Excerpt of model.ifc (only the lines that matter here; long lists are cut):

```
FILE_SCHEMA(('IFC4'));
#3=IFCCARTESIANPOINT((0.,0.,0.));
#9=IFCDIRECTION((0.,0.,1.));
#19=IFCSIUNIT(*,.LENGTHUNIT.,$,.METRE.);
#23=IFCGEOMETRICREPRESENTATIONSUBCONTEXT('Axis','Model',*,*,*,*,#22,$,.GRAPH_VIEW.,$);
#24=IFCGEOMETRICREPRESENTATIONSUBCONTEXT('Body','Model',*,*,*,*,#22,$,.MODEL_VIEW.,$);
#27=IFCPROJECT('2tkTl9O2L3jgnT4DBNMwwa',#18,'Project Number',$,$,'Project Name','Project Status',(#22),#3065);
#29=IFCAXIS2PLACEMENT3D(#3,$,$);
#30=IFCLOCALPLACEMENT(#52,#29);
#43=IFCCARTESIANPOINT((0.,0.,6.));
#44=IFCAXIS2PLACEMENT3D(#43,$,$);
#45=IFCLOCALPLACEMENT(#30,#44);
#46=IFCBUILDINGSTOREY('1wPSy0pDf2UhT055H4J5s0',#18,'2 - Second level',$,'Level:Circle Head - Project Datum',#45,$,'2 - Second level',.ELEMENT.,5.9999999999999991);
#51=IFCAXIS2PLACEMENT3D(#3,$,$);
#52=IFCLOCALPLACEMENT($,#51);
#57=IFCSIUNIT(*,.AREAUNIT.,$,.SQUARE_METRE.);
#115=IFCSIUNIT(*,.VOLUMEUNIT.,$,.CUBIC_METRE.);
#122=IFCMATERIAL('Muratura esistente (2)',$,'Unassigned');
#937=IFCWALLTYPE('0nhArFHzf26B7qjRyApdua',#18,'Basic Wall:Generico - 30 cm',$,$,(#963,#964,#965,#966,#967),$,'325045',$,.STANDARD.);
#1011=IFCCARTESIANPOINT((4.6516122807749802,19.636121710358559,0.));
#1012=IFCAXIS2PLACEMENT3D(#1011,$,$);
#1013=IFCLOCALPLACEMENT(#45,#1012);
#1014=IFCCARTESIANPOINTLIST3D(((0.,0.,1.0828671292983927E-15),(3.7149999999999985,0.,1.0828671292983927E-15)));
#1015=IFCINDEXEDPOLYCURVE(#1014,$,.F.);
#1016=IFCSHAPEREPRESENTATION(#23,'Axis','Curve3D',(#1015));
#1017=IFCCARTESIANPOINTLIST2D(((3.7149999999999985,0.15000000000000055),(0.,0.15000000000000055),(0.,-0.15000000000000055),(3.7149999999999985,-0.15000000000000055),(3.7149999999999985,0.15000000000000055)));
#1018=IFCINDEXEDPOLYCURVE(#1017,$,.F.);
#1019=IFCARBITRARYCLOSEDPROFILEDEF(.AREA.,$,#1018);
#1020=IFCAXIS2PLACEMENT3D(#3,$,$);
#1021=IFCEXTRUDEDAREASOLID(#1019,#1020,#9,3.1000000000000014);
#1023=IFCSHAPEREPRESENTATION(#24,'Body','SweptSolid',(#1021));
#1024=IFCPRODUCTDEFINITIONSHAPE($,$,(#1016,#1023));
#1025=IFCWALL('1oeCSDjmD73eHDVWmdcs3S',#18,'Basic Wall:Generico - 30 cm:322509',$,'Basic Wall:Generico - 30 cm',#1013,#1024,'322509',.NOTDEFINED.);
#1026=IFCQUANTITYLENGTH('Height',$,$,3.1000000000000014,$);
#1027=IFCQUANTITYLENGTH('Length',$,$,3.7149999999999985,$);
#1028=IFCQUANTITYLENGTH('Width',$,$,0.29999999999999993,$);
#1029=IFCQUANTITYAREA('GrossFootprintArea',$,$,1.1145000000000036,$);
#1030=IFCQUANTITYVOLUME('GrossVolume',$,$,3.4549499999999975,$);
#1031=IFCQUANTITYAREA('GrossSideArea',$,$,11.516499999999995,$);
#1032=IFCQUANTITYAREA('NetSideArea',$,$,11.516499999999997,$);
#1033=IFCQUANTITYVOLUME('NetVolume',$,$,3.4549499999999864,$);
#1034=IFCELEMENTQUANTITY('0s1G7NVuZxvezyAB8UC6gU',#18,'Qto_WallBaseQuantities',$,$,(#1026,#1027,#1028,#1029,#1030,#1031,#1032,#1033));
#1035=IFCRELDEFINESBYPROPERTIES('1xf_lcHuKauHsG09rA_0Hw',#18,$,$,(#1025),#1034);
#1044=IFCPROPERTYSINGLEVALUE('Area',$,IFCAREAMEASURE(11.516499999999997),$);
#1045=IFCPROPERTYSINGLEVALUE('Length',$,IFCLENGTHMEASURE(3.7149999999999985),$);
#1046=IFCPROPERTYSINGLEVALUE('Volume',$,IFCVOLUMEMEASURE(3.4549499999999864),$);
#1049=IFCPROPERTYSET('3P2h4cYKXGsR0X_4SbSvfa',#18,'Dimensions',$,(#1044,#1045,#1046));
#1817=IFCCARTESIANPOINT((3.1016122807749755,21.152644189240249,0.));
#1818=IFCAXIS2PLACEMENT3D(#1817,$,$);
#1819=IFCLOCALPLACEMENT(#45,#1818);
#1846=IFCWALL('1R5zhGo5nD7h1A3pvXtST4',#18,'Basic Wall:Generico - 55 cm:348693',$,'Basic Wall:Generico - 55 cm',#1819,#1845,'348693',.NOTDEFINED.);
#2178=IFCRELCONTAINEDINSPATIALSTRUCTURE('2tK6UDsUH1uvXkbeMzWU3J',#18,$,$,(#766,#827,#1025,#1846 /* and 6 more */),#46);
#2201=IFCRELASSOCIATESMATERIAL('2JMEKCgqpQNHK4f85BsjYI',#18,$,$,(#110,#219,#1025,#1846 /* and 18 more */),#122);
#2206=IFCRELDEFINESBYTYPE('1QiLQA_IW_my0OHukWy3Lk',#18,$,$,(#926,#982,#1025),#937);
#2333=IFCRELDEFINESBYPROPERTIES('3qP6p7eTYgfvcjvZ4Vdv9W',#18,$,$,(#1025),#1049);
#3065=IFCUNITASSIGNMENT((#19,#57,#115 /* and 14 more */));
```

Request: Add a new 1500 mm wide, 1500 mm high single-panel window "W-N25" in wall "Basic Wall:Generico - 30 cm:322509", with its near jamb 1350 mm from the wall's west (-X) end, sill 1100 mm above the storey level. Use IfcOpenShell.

```python
import numpy as np
import ifcopenshell
import ifcopenshell.api.feature
import ifcopenshell.api.geometry
import ifcopenshell.api.pset
import ifcopenshell.api.root
import ifcopenshell.api.spatial
import ifcopenshell.geom
import ifcopenshell.util.element
import ifcopenshell.util.placement
import ifcopenshell.util.representation
import ifcopenshell.util.shape
import ifcopenshell.util.unit

model = ifcopenshell.open("model.ifc")
unit_scale = ifcopenshell.util.unit.calculate_unit_scale(model)
area_scale = ifcopenshell.util.unit.calculate_unit_scale(model, "AREAUNIT")
volume_scale = ifcopenshell.util.unit.calculate_unit_scale(model, "VOLUMEUNIT")
settings = ifcopenshell.geom.settings()


def volume(element):
    """Net volume in cubic metres, openings subtracted."""
    shape = ifcopenshell.geom.create_shape(settings, element)
    return ifcopenshell.util.shape.get_volume(shape.geometry)


wall = model.by_guid("1oeCSDjmD73eHDVWmdcs3S")
storey = ifcopenshell.util.element.get_container(wall, ifc_class="IfcBuildingStorey")
context = ifcopenshell.util.representation.get_context(model, "Model", "Body", "MODEL_VIEW")
before = volume(wall)

width, height, from_end, sill = 1.5, 1.5, 1.35, 1.1  # metres

# The wall runs along its own X axis, and the end named is its -X end.
wall_shape = ifcopenshell.geom.create_shape(settings, wall)
x, y, z = ifcopenshell.util.shape.get_vertices(wall_shape.geometry).T
start = x.min() + from_end
face, thickness = float(y.min()), float(y.max() - y.min())
wall_matrix = ifcopenshell.util.placement.get_local_placement(wall.ObjectPlacement)
level = ifcopenshell.util.placement.get_local_placement(storey.ObjectPlacement)[2, 3]


def in_wall(x, y):
    """Placement at x, y metres in the wall's axes, at sill height."""
    matrix = wall_matrix.copy()
    matrix[:, 3] = wall_matrix @ np.array([x / unit_scale, y / unit_scale, 0.0, 1.0])
    matrix[2, 3] = level + sill / unit_scale
    return matrix


# Opening: a box that overshoots both wall faces by 50 mm.
opening = ifcopenshell.api.root.create_entity(model, ifc_class="IfcOpeningElement", predefined_type="OPENING")
box = ifcopenshell.api.geometry.add_wall_representation(
    model, context=context, length=width, height=height, thickness=thickness + 0.1
)
ifcopenshell.api.geometry.assign_representation(model, product=opening, representation=box)
ifcopenshell.api.geometry.edit_object_placement(model, product=opening, matrix=in_wall(start, face - 0.05), is_si=False)
ifcopenshell.api.feature.add_feature(model, feature=opening, element=wall)

window = ifcopenshell.api.root.create_entity(model, ifc_class="IfcWindow", name="W-N25", predefined_type="WINDOW")
window.OverallWidth, window.OverallHeight = width / unit_scale, height / unit_scale
window.PartitioningType = "SINGLE_PANEL"
body = ifcopenshell.api.geometry.add_window_representation(
    model,
    context=context,
    overall_width=window.OverallWidth,
    overall_height=window.OverallHeight,
    partition_type="SINGLE_PANEL",
)
ifcopenshell.api.geometry.assign_representation(model, product=window, representation=body)
ifcopenshell.api.spatial.assign_container(model, products=[window], relating_structure=storey)
ifcopenshell.api.feature.add_filling(model, opening=opening, element=window)

# Centre the window in the wall's thickness.
ifcopenshell.api.geometry.edit_object_placement(model, product=window, matrix=in_wall(start, face), is_si=False)
window_shape = ifcopenshell.geom.create_shape(settings, window)
depth = ifcopenshell.util.shape.get_vertices(window_shape.geometry)[:, 1]
offset = face + thickness / 2 - (depth.min() + depth.max()) / 2
ifcopenshell.api.geometry.edit_object_placement(model, product=window, matrix=in_wall(start, offset), is_si=False)

after = volume(wall)

# Update the wall's stored quantities.
qto = model.by_id(ifcopenshell.util.element.get_pset(wall, "Qto_WallBaseQuantities", should_inherit=False)["id"])
ifcopenshell.api.pset.edit_qto(model, qto=qto, properties={
    "NetSideArea": after / thickness / area_scale,
    "NetVolume": after / volume_scale,
})
pset = model.by_id(ifcopenshell.util.element.get_pset(wall, "Dimensions", should_inherit=False)["id"])
ifcopenshell.api.pset.edit_pset(model, pset=pset, properties={
    "Area": model.create_entity("IfcAreaMeasure", after / thickness / area_scale),
    "Volume": model.create_entity("IfcVolumeMeasure", after / volume_scale),
})

print(f"wall volume {before:.3f} -> {after:.3f} m3")

model.write("model_rev.ifc")
```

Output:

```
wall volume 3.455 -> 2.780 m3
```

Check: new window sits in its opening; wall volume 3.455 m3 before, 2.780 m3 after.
